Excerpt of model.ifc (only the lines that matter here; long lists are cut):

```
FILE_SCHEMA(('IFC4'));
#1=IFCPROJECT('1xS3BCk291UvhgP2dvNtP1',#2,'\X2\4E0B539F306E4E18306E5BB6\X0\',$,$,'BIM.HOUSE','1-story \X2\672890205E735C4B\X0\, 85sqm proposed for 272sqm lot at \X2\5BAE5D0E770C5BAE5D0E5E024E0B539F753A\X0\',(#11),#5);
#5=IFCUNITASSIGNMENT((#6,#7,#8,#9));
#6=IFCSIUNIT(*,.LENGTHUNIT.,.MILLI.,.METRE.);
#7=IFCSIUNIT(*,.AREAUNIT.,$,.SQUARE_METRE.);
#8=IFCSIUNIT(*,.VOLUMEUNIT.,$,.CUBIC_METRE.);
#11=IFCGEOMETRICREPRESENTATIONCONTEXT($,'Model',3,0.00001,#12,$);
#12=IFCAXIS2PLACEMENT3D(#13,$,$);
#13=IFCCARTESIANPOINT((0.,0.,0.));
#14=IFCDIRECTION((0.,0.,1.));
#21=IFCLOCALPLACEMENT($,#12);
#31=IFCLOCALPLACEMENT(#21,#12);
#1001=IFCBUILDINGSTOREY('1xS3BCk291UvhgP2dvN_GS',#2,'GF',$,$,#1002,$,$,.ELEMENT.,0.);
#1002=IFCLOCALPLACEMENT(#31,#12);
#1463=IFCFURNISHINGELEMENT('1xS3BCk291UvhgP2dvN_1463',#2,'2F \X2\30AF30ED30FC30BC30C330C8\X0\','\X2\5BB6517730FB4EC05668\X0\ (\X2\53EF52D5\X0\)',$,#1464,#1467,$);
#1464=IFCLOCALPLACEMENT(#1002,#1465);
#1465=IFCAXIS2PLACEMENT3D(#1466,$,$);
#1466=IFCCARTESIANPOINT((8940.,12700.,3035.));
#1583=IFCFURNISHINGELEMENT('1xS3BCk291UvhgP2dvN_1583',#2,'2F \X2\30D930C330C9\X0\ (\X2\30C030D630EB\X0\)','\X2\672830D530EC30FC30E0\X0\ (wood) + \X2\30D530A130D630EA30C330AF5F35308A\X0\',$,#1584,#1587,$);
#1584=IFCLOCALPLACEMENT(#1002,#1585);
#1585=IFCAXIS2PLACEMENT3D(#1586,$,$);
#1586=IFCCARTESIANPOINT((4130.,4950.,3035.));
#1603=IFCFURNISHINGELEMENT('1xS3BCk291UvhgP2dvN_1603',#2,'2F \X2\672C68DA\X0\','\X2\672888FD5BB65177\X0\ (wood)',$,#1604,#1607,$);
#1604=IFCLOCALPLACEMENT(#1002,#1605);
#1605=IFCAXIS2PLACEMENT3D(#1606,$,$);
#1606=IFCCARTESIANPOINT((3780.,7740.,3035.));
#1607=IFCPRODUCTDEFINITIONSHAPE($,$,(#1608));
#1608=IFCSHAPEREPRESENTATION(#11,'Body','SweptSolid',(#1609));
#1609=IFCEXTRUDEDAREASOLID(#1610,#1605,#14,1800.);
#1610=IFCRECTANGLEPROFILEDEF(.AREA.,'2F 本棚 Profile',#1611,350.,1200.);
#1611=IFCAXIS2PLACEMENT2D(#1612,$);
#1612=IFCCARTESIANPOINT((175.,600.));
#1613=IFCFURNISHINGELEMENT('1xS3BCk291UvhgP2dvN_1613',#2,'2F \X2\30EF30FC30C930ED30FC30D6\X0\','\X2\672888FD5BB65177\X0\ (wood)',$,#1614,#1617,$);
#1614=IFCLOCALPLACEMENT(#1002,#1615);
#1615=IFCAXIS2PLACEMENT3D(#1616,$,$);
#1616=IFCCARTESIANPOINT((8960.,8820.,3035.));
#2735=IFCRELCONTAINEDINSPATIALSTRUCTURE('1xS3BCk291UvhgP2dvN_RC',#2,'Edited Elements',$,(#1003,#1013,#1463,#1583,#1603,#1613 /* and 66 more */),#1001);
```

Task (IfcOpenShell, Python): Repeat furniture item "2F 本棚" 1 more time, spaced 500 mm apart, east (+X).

```python
import numpy as np
import ifcopenshell
import ifcopenshell.api.geometry
import ifcopenshell.api.root
import ifcopenshell.util.element
import ifcopenshell.util.placement
import ifcopenshell.util.unit

model = ifcopenshell.open("model.ifc")
unit_scale = ifcopenshell.util.unit.calculate_unit_scale(model)


def reuse_history(source, copy):
    """copy_class also copies each property set's owner history, people and application; keep the originals."""
    for rel in copy.IsDefinedBy:
        if rel.is_a("IfcRelDefinesByProperties") and (history := rel.RelatingPropertyDefinition.OwnerHistory):
            rel.RelatingPropertyDefinition.OwnerHistory = source.OwnerHistory
            ifcopenshell.util.element.remove_deep2(model, history)


source = model.by_id(1603)
base = ifcopenshell.util.placement.get_local_placement(source.ObjectPlacement)
step = np.array([1.0, 0.0, 0.0]) * 0.5 / unit_scale

for i in range(1, 2):
    copy = ifcopenshell.api.root.copy_class(model, product=source)
    copy.Representation = ifcopenshell.util.element.copy_deep(
        model, source.Representation, exclude=["IfcGeometricRepresentationContext", "IfcRepresentationMap"]
    )
    reuse_history(source, copy)
    matrix = base.copy()
    matrix[:3, 3] += i * step
    print("added at", matrix[:3, 3].round(3) + 0.0)
    ifcopenshell.api.geometry.edit_object_placement(model, product=copy, matrix=matrix, is_si=False)

model.write("model-out.ifc")
```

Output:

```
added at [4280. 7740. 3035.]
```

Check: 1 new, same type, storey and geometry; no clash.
